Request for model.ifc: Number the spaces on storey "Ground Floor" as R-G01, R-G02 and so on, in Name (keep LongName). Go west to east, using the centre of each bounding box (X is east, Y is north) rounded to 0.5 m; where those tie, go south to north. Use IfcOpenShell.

First a look at what the model holds.

```python
import ifcopenshell
import ifcopenshell.util.element
import ifcopenshell.util.placement

model = ifcopenshell.open("model.ifc")
print(model.schema)
storey = next(s for s in model.by_type("IfcBuildingStorey") if s.Name == "Ground Floor")
spaces = [e for e in ifcopenshell.util.element.get_decomposition(storey) if e.is_a("IfcSpace")]
for e in sorted(spaces, key=lambda e: e.id()):
    origin = ifcopenshell.util.placement.get_local_placement(e.ObjectPlacement)[:3, 3]
    print(e.id(), e.Name, e.LongName, origin.round(2) + 0.0, sep=" | ")
```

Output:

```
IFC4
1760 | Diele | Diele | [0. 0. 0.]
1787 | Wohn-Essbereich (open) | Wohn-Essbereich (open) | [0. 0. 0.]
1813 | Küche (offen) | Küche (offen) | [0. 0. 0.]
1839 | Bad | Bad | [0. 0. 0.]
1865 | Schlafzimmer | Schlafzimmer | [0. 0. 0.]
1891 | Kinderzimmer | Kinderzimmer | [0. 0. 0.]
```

```python
import ifcopenshell
import ifcopenshell.geom
import ifcopenshell.util.element
import ifcopenshell.util.shape

model = ifcopenshell.open("model.ifc")
settings = ifcopenshell.geom.settings()
settings.set("use-world-coords", True)


def centre(element):
    shape = ifcopenshell.geom.create_shape(settings, element)
    return ifcopenshell.util.shape.get_bbox_centroid(shape.geometry)


storey = next(s for s in model.by_type("IfcBuildingStorey") if s.Name == "Ground Floor")
spaces = [e for e in ifcopenshell.util.element.get_decomposition(storey) if e.is_a("IfcSpace")]

# Insertion points can sit at a corner or the storey origin, so sort by the geometry (in metres).
centres = {e: centre(e) for e in spaces}
spaces.sort(key=lambda e: (round(centres[e][0] / 0.5), centres[e][1]))

for i, e in enumerate(spaces, start=1):
    number = f"R-G{i:02d}"
    e.Name = number
    print(e.id(), number)

model.write("model_updated.ifc")
```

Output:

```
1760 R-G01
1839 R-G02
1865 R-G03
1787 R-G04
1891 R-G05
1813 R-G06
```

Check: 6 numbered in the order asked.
